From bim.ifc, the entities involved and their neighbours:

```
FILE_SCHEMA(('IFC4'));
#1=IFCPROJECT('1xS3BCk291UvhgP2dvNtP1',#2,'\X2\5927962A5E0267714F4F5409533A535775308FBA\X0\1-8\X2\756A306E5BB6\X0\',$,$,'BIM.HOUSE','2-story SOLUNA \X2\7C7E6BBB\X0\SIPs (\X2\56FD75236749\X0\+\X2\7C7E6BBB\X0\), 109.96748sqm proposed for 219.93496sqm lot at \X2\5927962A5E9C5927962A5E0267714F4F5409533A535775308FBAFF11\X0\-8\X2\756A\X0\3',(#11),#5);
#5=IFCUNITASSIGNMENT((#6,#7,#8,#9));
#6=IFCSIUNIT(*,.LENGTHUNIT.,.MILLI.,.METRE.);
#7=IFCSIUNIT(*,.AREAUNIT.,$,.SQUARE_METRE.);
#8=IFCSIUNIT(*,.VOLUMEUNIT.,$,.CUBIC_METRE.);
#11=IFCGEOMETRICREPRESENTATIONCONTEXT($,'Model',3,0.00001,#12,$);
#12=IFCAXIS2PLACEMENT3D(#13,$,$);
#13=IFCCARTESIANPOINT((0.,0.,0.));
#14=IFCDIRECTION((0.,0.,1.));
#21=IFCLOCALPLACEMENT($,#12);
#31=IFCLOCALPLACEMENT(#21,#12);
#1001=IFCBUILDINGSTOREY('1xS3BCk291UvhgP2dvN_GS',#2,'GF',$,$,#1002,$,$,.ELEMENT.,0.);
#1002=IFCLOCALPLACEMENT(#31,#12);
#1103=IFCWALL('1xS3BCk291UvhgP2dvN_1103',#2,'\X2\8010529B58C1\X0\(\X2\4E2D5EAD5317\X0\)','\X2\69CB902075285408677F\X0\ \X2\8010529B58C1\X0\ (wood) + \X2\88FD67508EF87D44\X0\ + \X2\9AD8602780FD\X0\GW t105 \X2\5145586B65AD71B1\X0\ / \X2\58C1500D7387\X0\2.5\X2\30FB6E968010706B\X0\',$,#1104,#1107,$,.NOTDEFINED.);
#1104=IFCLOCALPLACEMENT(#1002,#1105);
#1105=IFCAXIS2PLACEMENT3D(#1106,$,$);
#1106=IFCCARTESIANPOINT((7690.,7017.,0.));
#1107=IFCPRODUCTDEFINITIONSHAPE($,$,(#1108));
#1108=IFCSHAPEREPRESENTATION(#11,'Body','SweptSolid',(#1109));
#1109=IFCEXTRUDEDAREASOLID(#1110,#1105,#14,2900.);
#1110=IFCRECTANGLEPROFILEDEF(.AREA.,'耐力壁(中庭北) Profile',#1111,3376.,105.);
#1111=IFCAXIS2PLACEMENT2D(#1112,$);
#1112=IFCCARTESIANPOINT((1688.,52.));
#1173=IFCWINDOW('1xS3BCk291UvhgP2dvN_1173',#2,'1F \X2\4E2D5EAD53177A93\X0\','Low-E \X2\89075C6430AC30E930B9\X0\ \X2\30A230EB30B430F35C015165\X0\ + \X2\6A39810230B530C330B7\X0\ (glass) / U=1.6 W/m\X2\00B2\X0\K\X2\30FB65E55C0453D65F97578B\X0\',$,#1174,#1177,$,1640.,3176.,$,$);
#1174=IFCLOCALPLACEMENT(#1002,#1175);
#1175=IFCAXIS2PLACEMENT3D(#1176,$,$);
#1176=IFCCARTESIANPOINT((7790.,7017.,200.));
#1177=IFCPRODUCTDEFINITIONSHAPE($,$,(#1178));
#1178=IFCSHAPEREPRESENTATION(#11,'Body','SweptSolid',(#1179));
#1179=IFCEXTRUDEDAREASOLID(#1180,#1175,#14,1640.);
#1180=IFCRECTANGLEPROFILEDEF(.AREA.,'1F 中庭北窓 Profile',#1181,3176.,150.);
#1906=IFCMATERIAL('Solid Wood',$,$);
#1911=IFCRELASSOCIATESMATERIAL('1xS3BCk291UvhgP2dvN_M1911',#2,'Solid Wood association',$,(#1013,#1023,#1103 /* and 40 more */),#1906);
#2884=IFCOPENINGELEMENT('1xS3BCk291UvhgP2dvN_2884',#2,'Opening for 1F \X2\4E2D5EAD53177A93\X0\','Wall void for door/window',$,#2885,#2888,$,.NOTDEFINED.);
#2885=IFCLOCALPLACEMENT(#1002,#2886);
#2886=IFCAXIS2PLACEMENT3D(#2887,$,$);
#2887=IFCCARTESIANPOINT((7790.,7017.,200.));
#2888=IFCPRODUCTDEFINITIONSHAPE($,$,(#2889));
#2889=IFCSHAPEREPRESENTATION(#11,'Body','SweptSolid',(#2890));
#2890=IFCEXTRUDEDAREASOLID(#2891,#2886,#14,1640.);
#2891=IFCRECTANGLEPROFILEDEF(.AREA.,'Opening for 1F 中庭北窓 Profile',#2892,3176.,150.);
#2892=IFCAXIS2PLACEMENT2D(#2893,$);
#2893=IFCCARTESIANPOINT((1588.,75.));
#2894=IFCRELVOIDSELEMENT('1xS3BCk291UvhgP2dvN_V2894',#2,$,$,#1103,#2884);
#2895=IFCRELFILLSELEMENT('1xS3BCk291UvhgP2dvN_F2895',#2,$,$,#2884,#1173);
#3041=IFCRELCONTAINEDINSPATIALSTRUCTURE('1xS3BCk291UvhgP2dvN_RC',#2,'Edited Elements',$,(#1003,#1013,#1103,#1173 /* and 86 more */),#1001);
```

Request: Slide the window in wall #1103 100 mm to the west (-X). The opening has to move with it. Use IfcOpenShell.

```python
import ifcopenshell
import ifcopenshell.api.geometry
import ifcopenshell.util.placement

model = ifcopenshell.open("bim.ifc")

window = model.by_id(1173)
opening = window.FillsVoids[0].RelatingOpeningElement
wall = opening.VoidsElements[0].RelatingBuildingElement

wall_matrix = ifcopenshell.util.placement.get_local_placement(wall.ObjectPlacement)
shift = wall_matrix[:3, 0] * -100.0
before = ifcopenshell.util.placement.get_local_placement(window.ObjectPlacement)[:3, 3].copy()

# The window is not placed relative to its opening, so move both.
for product in (opening, window):
    matrix = ifcopenshell.util.placement.get_local_placement(product.ObjectPlacement)
    matrix[:3, 3] += shift
    ifcopenshell.api.geometry.edit_object_placement(model, product=product, matrix=matrix, is_si=False)

after = ifcopenshell.util.placement.get_local_placement(window.ObjectPlacement)[:3, 3]
print("window moved by", (after - before).round(3) + 0.0)

model.write("bim_edited.ifc")
```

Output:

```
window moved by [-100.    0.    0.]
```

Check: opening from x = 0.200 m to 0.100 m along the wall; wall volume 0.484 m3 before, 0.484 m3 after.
